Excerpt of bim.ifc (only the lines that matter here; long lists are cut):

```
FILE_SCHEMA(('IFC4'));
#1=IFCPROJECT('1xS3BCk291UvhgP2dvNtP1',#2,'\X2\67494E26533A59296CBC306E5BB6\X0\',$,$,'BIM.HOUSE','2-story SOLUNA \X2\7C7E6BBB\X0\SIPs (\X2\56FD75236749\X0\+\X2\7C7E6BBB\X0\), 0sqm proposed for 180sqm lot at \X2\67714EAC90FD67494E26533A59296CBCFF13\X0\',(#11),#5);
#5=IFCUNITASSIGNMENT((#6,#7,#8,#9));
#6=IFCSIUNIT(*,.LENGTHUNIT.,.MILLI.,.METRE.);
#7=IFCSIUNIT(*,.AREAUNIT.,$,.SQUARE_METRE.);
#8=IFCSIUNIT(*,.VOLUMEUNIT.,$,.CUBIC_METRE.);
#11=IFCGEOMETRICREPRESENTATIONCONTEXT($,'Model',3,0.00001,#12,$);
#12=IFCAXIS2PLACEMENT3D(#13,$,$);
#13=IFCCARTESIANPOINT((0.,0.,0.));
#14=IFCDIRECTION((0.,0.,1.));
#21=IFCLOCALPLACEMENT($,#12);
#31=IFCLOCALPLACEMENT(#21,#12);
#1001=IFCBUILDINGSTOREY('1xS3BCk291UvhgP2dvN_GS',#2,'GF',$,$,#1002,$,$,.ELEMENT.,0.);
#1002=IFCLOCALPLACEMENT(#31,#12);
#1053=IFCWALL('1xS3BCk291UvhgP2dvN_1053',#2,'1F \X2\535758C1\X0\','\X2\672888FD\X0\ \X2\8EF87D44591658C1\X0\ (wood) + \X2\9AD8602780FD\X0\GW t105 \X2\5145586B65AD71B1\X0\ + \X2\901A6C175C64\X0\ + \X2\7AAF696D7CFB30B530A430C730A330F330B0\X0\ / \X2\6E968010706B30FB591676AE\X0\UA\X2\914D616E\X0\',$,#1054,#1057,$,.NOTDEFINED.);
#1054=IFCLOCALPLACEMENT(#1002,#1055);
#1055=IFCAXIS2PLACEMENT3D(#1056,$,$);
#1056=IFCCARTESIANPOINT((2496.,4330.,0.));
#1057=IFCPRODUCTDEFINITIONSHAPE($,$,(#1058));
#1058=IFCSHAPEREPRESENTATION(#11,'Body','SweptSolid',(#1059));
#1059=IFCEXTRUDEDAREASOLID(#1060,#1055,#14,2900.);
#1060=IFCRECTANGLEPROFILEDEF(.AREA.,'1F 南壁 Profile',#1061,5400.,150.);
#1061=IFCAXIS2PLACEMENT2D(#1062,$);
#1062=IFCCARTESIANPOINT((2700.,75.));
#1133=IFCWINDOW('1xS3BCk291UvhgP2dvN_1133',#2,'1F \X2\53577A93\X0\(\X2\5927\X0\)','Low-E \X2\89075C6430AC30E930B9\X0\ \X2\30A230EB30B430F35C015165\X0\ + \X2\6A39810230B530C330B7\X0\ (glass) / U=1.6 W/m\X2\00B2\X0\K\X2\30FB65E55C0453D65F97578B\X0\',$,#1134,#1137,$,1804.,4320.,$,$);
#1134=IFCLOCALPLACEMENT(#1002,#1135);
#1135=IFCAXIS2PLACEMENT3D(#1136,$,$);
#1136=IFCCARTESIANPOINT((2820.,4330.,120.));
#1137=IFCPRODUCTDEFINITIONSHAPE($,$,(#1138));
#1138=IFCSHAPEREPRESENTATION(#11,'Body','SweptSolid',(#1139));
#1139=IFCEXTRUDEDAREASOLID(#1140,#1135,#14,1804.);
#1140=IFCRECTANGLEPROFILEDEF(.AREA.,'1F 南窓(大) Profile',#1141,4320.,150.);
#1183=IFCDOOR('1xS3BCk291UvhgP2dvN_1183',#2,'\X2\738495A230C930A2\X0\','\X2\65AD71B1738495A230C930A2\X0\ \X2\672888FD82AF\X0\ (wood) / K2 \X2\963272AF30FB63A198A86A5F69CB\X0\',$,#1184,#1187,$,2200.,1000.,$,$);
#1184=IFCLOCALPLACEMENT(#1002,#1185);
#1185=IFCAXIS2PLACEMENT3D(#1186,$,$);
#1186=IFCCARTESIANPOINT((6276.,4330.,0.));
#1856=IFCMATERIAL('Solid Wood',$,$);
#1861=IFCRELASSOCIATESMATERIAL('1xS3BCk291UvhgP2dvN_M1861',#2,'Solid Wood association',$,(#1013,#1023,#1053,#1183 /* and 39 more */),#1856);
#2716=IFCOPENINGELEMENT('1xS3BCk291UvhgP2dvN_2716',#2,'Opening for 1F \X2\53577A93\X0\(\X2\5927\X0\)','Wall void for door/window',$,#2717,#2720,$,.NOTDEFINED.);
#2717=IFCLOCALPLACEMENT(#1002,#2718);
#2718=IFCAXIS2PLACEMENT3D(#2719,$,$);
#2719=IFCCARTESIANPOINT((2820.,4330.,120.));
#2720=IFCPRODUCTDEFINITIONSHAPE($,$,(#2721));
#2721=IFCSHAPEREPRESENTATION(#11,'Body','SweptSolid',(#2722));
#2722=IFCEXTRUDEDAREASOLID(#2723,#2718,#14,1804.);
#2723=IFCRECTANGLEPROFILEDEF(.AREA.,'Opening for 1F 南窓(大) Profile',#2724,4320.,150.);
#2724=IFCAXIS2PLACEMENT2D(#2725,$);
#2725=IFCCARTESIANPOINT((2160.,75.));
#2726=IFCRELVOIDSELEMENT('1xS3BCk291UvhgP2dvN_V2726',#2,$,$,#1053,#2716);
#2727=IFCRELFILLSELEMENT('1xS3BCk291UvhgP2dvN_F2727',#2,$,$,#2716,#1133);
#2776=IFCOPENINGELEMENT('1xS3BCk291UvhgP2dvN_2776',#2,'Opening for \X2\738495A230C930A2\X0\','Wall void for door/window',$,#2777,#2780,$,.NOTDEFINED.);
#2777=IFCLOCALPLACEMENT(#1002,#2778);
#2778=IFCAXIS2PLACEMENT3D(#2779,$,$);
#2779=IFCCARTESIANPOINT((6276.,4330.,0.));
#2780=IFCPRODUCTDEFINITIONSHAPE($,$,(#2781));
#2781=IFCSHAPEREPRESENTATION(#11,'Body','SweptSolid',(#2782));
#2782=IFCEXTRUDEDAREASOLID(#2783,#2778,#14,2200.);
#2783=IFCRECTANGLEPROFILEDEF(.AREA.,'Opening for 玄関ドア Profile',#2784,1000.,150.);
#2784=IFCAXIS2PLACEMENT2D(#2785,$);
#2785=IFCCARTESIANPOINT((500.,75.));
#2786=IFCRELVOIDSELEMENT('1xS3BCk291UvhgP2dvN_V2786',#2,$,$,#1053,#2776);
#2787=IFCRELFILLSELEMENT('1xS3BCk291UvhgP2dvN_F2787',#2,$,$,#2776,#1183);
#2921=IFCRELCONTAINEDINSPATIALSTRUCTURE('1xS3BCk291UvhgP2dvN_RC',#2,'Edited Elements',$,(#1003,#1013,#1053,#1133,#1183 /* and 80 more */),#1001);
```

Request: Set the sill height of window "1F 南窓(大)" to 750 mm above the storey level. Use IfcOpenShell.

```python
import numpy as np
import ifcopenshell
import ifcopenshell.api.geometry
import ifcopenshell.geom
import ifcopenshell.util.element
import ifcopenshell.util.placement
import ifcopenshell.util.shape
import ifcopenshell.util.unit

model = ifcopenshell.open("bim.ifc")
unit_scale = ifcopenshell.util.unit.calculate_unit_scale(model)

window = model.by_id(1133)
opening = window.FillsVoids[0].RelatingOpeningElement
storey = ifcopenshell.util.element.get_container(window, ifc_class="IfcBuildingStorey")
level = ifcopenshell.util.placement.get_local_placement(storey.ObjectPlacement)[2, 3]

# The opening's origin need not be at the sill, so measure its lowest point.
shape = ifcopenshell.geom.create_shape(ifcopenshell.geom.settings(), opening)
bottom = ifcopenshell.util.shape.get_shape_bottom_elevation(shape, shape.geometry) / unit_scale
dz = level + 0.75 / unit_scale - bottom

shift = np.array([0.0, 0.0, dz])
# The window is not placed relative to its opening, so move both.
for product in (opening, window):
    matrix = ifcopenshell.util.placement.get_local_placement(product.ObjectPlacement)
    matrix[:3, 3] += shift
    ifcopenshell.api.geometry.edit_object_placement(model, product=product, matrix=matrix, is_si=False)

print(f"moved by {dz * unit_scale:+.3f} m")

model.write("bim_rev.ifc")
```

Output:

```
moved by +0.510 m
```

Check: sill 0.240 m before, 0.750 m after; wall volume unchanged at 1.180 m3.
